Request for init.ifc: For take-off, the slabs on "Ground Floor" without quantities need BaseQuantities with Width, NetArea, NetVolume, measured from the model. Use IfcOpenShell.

First a look at what the model holds.

```python
import ifcopenshell
import ifcopenshell.util.element
import ifcopenshell.util.unit

model = ifcopenshell.open("init.ifc")
print(model.schema)
for unit_type in ("LENGTHUNIT", "AREAUNIT", "VOLUMEUNIT"):
    print(unit_type, ifcopenshell.util.unit.calculate_unit_scale(model, unit_type))
storey = next(s for s in model.by_type("IfcBuildingStorey") if s.Name == "Ground Floor")
slabs = [e for e in ifcopenshell.util.element.get_decomposition(storey) if e.is_a("IfcSlab")]
for e in sorted(slabs, key=lambda e: e.id()):
    print(e.id(), e.is_a(), e.Name, list(ifcopenshell.util.element.get_psets(e, qtos_only=True)), sep=" | ")
```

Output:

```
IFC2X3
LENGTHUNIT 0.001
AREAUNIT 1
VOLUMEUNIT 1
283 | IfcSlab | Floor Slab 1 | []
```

```python
import ifcopenshell
import ifcopenshell.api.pset
import ifcopenshell.geom
import ifcopenshell.util.element
import ifcopenshell.util.shape
import ifcopenshell.util.unit

model = ifcopenshell.open("init.ifc")
unit_scale = ifcopenshell.util.unit.calculate_unit_scale(model)
area_scale = ifcopenshell.util.unit.calculate_unit_scale(model, "AREAUNIT")
volume_scale = ifcopenshell.util.unit.calculate_unit_scale(model, "VOLUMEUNIT")
settings = ifcopenshell.geom.settings()

storey = next(s for s in model.by_type("IfcBuildingStorey") if s.Name == "Ground Floor")
slabs = [e for e in ifcopenshell.util.element.get_decomposition(storey) if e.is_a("IfcSlab")]

for e in sorted(slabs, key=lambda e: e.id()):
    if ifcopenshell.util.element.get_psets(e, qtos_only=True, should_inherit=False):
        continue
    # Geometry comes back in metres, in the element's own axes.
    shape = ifcopenshell.geom.create_shape(settings, e)
    values = {
        "Width": ifcopenshell.util.shape.get_z(shape.geometry) / unit_scale,
        "NetArea": ifcopenshell.util.shape.get_footprint_area(shape.geometry) / area_scale,
        "NetVolume": ifcopenshell.util.shape.get_volume(shape.geometry) / volume_scale,
    }
    qto = ifcopenshell.api.pset.add_qto(model, product=e, name="BaseQuantities")
    ifcopenshell.api.pset.edit_qto(model, qto=qto, properties=values)
    print(e.id(), {k: round(v, 3) for k, v in values.items()})

model.write("init_rev.ifc")
```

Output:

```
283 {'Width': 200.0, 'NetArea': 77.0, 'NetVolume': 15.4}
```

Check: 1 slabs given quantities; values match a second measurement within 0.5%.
